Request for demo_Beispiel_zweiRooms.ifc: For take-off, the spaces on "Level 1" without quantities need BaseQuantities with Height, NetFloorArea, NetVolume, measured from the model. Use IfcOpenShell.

First a look at what the model holds.

```python
import ifcopenshell
import ifcopenshell.util.element
import ifcopenshell.util.unit

model = ifcopenshell.open("demo_Beispiel_zweiRooms.ifc")
print(model.schema)
for unit_type in ("LENGTHUNIT", "AREAUNIT", "VOLUMEUNIT"):
    print(unit_type, ifcopenshell.util.unit.calculate_unit_scale(model, unit_type))
storey = next(s for s in model.by_type("IfcBuildingStorey") if s.Name == "Level 1")
spaces = [e for e in ifcopenshell.util.element.get_decomposition(storey) if e.is_a("IfcSpace")]
for e in sorted(spaces, key=lambda e: e.id()):
    print(e.id(), e.is_a(), e.Name, list(ifcopenshell.util.element.get_psets(e, qtos_only=True)), sep=" | ")
```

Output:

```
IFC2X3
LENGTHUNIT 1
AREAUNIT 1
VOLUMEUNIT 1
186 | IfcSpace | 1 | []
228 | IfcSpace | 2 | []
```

```python
import ifcopenshell
import ifcopenshell.api.pset
import ifcopenshell.geom
import ifcopenshell.util.element
import ifcopenshell.util.shape
import ifcopenshell.util.unit

model = ifcopenshell.open("demo_Beispiel_zweiRooms.ifc")
unit_scale = ifcopenshell.util.unit.calculate_unit_scale(model)
area_scale = ifcopenshell.util.unit.calculate_unit_scale(model, "AREAUNIT")
volume_scale = ifcopenshell.util.unit.calculate_unit_scale(model, "VOLUMEUNIT")
settings = ifcopenshell.geom.settings()

storey = next(s for s in model.by_type("IfcBuildingStorey") if s.Name == "Level 1")
spaces = [e for e in ifcopenshell.util.element.get_decomposition(storey) if e.is_a("IfcSpace")]

for e in sorted(spaces, key=lambda e: e.id()):
    if ifcopenshell.util.element.get_psets(e, qtos_only=True, should_inherit=False):
        continue
    # Geometry comes back in metres, in the element's own axes.
    shape = ifcopenshell.geom.create_shape(settings, e)
    values = {
        "Height": ifcopenshell.util.shape.get_z(shape.geometry) / unit_scale,
        "NetFloorArea": ifcopenshell.util.shape.get_footprint_area(shape.geometry) / area_scale,
        "NetVolume": ifcopenshell.util.shape.get_volume(shape.geometry) / volume_scale,
    }
    qto = ifcopenshell.api.pset.add_qto(model, product=e, name="BaseQuantities")
    ifcopenshell.api.pset.edit_qto(model, qto=qto, properties=values)
    print(e.id(), {k: round(v, 3) for k, v in values.items()})

model.write("demo_Beispiel_zweiRooms-out.ifc")
```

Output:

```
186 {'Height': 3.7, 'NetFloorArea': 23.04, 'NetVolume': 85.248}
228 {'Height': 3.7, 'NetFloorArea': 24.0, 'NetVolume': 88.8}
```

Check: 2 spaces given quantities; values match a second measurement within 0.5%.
